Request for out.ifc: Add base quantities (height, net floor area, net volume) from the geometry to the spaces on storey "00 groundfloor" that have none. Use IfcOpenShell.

First a look at what the model holds.

```python
import ifcopenshell
import ifcopenshell.util.element
import ifcopenshell.util.unit

model = ifcopenshell.open("out.ifc")
print(model.schema)
for unit_type in ("LENGTHUNIT", "AREAUNIT", "VOLUMEUNIT"):
    print(unit_type, ifcopenshell.util.unit.calculate_unit_scale(model, unit_type))
storey = next(s for s in model.by_type("IfcBuildingStorey") if s.Name == "00 groundfloor")
spaces = [e for e in ifcopenshell.util.element.get_decomposition(storey) if e.is_a("IfcSpace")]
for e in sorted(spaces, key=lambda e: e.id()):
    print(e.id(), e.is_a(), e.Name, list(ifcopenshell.util.element.get_psets(e, qtos_only=True)), sep=" | ")
```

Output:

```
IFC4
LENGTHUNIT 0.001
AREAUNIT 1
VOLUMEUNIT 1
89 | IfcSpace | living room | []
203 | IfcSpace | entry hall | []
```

```python
import ifcopenshell
import ifcopenshell.api.pset
import ifcopenshell.geom
import ifcopenshell.util.element
import ifcopenshell.util.shape
import ifcopenshell.util.unit

model = ifcopenshell.open("out.ifc")
unit_scale = ifcopenshell.util.unit.calculate_unit_scale(model)
area_scale = ifcopenshell.util.unit.calculate_unit_scale(model, "AREAUNIT")
volume_scale = ifcopenshell.util.unit.calculate_unit_scale(model, "VOLUMEUNIT")
settings = ifcopenshell.geom.settings()

storey = next(s for s in model.by_type("IfcBuildingStorey") if s.Name == "00 groundfloor")
spaces = [e for e in ifcopenshell.util.element.get_decomposition(storey) if e.is_a("IfcSpace")]

for e in sorted(spaces, key=lambda e: e.id()):
    if ifcopenshell.util.element.get_psets(e, qtos_only=True, should_inherit=False):
        continue
    # Geometry comes back in metres, in the element's own axes.
    shape = ifcopenshell.geom.create_shape(settings, e)
    values = {
        "Height": ifcopenshell.util.shape.get_z(shape.geometry) / unit_scale,
        "NetFloorArea": ifcopenshell.util.shape.get_footprint_area(shape.geometry) / area_scale,
        "NetVolume": ifcopenshell.util.shape.get_volume(shape.geometry) / volume_scale,
    }
    qto = ifcopenshell.api.pset.add_qto(model, product=e, name="Qto_SpaceBaseQuantities")
    ifcopenshell.api.pset.edit_qto(model, qto=qto, properties=values)
    print(e.id(), {k: round(v, 3) for k, v in values.items()})

model.write("out_v2.ifc")
```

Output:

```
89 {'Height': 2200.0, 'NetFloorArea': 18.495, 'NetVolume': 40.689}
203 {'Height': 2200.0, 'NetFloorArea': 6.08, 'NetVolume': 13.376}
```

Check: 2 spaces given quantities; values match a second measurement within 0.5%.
